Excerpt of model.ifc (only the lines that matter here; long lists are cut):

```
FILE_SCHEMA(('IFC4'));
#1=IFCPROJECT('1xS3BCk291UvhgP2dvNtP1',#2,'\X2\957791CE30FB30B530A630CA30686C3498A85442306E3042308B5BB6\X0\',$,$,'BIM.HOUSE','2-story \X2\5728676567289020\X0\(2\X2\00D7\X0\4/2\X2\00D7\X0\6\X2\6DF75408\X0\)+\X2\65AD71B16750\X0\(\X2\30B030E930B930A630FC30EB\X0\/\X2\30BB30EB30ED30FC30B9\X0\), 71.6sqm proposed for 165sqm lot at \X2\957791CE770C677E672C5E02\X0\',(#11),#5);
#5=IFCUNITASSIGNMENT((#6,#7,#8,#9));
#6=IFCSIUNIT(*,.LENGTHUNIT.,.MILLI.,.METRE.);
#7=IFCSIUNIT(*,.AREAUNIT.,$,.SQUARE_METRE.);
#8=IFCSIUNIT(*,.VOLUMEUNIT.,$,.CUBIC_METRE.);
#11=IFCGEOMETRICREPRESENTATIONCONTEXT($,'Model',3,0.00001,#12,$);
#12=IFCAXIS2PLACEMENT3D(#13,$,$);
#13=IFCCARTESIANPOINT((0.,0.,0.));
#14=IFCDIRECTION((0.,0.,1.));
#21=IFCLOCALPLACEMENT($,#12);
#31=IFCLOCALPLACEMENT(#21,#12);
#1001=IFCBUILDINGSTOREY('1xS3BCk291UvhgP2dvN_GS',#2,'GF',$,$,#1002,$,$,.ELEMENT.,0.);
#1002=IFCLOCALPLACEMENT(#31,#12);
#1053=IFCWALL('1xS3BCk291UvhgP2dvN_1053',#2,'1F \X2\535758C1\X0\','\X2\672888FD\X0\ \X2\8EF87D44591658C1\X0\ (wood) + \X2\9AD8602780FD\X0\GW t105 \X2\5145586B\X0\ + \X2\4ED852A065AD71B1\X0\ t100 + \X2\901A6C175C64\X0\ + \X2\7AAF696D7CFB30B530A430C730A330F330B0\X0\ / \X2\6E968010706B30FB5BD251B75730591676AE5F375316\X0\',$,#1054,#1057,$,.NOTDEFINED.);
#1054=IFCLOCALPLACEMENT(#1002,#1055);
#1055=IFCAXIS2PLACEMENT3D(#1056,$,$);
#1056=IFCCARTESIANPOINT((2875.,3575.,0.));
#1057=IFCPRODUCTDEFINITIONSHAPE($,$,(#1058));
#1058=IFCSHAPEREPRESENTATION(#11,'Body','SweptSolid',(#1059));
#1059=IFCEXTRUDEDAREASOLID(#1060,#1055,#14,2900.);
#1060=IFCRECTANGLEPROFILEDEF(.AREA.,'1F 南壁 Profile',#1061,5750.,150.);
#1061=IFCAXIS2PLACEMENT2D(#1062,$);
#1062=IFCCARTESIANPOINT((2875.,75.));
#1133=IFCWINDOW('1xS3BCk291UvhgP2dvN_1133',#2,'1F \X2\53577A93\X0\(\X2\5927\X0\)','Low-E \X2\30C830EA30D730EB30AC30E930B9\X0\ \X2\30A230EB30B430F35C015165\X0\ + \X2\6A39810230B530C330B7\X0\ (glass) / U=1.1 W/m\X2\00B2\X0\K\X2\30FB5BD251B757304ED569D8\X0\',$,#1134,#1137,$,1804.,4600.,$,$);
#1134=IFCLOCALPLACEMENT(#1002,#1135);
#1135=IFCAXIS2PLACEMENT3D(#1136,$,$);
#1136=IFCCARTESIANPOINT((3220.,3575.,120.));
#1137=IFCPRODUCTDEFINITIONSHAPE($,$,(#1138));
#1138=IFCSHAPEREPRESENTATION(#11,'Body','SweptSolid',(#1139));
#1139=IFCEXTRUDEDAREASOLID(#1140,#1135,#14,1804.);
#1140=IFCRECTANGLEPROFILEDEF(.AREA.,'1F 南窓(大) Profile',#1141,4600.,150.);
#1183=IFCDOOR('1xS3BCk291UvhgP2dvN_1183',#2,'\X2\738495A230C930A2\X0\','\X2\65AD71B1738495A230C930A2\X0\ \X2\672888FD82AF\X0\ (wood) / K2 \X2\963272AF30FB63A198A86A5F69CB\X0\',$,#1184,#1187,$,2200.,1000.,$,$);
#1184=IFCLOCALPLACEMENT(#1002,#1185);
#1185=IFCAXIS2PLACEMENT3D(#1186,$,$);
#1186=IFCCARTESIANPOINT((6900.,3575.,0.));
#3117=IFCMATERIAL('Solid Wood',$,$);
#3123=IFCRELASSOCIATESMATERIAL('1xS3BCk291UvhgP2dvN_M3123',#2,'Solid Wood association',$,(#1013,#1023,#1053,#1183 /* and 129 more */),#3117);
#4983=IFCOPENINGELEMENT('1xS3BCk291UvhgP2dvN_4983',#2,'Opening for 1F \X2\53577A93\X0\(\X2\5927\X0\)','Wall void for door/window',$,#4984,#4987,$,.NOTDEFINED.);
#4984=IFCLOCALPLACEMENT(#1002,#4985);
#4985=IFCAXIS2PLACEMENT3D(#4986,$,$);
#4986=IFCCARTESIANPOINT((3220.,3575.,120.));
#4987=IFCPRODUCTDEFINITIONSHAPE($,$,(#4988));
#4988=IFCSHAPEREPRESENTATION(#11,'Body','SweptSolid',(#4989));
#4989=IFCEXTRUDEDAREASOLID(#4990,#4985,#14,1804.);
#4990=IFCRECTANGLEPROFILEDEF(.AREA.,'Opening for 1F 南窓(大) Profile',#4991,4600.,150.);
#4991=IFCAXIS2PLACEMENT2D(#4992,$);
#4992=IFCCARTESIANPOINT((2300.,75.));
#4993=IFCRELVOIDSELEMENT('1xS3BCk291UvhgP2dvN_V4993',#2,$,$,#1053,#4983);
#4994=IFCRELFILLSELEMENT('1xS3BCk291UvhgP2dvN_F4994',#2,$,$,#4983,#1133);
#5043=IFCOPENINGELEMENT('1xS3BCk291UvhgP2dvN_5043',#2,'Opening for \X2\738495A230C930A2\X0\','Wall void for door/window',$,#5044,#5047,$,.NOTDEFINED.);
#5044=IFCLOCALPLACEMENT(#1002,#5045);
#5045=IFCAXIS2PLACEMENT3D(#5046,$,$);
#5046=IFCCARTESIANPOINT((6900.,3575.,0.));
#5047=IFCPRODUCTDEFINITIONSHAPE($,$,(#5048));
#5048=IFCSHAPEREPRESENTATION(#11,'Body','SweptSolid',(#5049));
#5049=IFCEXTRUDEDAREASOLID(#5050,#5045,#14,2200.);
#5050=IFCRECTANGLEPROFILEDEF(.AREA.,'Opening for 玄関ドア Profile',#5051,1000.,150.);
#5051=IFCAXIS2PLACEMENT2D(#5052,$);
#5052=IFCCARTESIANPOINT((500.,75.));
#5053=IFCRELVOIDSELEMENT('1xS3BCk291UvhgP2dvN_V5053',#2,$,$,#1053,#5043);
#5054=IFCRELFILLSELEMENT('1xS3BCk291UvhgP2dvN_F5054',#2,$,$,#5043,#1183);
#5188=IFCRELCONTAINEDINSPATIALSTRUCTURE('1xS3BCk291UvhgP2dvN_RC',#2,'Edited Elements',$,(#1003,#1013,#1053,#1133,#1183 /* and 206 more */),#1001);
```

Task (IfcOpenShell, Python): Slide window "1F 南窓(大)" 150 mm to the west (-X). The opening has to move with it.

```python
import ifcopenshell
import ifcopenshell.api.geometry
import ifcopenshell.util.placement

model = ifcopenshell.open("model.ifc")

window = model.by_guid("1xS3BCk291UvhgP2dvN_1133")
opening = window.FillsVoids[0].RelatingOpeningElement
wall = opening.VoidsElements[0].RelatingBuildingElement

wall_matrix = ifcopenshell.util.placement.get_local_placement(wall.ObjectPlacement)
shift = wall_matrix[:3, 0] * -150.0
before = ifcopenshell.util.placement.get_local_placement(window.ObjectPlacement)[:3, 3].copy()

# The window is not placed relative to its opening, so move both.
for product in (opening, window):
    matrix = ifcopenshell.util.placement.get_local_placement(product.ObjectPlacement)
    matrix[:3, 3] += shift
    ifcopenshell.api.geometry.edit_object_placement(model, product=product, matrix=matrix, is_si=False)

after = ifcopenshell.util.placement.get_local_placement(window.ObjectPlacement)[:3, 3]
print("window moved by", (after - before).round(3) + 0.0)

model.write("model_edited.ifc")
```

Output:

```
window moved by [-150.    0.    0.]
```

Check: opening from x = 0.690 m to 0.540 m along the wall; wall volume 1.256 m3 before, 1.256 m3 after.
